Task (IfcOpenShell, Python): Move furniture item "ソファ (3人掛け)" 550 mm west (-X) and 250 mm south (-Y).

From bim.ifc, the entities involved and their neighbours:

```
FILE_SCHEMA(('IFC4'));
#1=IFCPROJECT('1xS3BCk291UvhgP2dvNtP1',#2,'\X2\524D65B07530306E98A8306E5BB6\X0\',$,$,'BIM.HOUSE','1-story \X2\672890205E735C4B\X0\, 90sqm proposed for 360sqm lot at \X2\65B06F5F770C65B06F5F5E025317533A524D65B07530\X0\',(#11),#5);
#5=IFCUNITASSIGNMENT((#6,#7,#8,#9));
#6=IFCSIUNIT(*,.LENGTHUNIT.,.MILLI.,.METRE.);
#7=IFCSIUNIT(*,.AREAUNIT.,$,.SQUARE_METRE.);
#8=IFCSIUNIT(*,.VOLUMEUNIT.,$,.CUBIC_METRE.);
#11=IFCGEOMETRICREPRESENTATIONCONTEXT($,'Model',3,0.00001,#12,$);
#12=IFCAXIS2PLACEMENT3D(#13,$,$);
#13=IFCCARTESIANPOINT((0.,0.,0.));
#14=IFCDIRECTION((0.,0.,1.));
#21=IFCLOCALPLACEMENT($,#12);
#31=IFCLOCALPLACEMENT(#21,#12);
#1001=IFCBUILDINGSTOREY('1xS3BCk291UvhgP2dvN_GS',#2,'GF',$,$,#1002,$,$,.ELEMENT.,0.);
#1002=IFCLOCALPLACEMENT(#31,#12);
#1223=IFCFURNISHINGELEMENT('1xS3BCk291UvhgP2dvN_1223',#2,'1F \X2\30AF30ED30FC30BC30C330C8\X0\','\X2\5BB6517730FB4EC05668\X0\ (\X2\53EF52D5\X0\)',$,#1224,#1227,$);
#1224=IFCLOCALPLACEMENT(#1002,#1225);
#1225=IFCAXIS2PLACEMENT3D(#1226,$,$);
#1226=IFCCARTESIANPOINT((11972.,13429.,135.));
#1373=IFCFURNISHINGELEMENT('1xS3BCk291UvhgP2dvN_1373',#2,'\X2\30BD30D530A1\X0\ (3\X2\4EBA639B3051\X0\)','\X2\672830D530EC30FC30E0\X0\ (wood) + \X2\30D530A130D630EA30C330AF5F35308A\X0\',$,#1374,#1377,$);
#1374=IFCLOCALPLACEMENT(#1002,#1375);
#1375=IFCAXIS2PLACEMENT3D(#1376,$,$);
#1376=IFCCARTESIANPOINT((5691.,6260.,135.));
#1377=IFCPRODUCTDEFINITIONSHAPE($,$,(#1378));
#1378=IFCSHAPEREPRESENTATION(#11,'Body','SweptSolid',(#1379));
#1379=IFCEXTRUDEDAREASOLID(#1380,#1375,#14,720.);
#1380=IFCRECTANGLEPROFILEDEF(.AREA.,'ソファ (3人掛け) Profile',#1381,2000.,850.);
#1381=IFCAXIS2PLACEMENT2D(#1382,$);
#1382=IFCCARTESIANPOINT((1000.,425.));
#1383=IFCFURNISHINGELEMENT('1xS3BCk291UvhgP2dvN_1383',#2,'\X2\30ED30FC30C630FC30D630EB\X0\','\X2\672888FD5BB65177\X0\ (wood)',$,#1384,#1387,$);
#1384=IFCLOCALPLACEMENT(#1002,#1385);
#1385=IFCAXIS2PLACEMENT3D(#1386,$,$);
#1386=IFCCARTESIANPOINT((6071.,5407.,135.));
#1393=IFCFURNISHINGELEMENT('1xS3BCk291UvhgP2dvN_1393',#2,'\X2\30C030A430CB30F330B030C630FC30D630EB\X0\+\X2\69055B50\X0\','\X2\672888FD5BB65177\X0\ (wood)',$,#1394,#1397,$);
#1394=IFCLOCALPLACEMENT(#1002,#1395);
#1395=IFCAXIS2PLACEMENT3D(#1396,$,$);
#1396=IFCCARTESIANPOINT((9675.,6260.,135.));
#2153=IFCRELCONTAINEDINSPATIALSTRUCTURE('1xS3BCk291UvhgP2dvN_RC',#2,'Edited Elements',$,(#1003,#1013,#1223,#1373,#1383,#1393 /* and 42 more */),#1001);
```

```python
import ifcopenshell
import ifcopenshell.api.geometry
import ifcopenshell.util.placement
import ifcopenshell.util.unit

model = ifcopenshell.open("bim.ifc")
unit_scale = ifcopenshell.util.unit.calculate_unit_scale(model)

item = model.by_guid("1xS3BCk291UvhgP2dvN_1373")
matrix = ifcopenshell.util.placement.get_local_placement(item.ObjectPlacement)
matrix[0, 3] -= 0.55 / unit_scale
matrix[1, 3] -= 0.25 / unit_scale
ifcopenshell.api.geometry.edit_object_placement(model, product=item, matrix=matrix, is_si=False)

print(ifcopenshell.util.placement.get_local_placement(item.ObjectPlacement).round(3) + 0.0)

model.write("bim-out.ifc")
```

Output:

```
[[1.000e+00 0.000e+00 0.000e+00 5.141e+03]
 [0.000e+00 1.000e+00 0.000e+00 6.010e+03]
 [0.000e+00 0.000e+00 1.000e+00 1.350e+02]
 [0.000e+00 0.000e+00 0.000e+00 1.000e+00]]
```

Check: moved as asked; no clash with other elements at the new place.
